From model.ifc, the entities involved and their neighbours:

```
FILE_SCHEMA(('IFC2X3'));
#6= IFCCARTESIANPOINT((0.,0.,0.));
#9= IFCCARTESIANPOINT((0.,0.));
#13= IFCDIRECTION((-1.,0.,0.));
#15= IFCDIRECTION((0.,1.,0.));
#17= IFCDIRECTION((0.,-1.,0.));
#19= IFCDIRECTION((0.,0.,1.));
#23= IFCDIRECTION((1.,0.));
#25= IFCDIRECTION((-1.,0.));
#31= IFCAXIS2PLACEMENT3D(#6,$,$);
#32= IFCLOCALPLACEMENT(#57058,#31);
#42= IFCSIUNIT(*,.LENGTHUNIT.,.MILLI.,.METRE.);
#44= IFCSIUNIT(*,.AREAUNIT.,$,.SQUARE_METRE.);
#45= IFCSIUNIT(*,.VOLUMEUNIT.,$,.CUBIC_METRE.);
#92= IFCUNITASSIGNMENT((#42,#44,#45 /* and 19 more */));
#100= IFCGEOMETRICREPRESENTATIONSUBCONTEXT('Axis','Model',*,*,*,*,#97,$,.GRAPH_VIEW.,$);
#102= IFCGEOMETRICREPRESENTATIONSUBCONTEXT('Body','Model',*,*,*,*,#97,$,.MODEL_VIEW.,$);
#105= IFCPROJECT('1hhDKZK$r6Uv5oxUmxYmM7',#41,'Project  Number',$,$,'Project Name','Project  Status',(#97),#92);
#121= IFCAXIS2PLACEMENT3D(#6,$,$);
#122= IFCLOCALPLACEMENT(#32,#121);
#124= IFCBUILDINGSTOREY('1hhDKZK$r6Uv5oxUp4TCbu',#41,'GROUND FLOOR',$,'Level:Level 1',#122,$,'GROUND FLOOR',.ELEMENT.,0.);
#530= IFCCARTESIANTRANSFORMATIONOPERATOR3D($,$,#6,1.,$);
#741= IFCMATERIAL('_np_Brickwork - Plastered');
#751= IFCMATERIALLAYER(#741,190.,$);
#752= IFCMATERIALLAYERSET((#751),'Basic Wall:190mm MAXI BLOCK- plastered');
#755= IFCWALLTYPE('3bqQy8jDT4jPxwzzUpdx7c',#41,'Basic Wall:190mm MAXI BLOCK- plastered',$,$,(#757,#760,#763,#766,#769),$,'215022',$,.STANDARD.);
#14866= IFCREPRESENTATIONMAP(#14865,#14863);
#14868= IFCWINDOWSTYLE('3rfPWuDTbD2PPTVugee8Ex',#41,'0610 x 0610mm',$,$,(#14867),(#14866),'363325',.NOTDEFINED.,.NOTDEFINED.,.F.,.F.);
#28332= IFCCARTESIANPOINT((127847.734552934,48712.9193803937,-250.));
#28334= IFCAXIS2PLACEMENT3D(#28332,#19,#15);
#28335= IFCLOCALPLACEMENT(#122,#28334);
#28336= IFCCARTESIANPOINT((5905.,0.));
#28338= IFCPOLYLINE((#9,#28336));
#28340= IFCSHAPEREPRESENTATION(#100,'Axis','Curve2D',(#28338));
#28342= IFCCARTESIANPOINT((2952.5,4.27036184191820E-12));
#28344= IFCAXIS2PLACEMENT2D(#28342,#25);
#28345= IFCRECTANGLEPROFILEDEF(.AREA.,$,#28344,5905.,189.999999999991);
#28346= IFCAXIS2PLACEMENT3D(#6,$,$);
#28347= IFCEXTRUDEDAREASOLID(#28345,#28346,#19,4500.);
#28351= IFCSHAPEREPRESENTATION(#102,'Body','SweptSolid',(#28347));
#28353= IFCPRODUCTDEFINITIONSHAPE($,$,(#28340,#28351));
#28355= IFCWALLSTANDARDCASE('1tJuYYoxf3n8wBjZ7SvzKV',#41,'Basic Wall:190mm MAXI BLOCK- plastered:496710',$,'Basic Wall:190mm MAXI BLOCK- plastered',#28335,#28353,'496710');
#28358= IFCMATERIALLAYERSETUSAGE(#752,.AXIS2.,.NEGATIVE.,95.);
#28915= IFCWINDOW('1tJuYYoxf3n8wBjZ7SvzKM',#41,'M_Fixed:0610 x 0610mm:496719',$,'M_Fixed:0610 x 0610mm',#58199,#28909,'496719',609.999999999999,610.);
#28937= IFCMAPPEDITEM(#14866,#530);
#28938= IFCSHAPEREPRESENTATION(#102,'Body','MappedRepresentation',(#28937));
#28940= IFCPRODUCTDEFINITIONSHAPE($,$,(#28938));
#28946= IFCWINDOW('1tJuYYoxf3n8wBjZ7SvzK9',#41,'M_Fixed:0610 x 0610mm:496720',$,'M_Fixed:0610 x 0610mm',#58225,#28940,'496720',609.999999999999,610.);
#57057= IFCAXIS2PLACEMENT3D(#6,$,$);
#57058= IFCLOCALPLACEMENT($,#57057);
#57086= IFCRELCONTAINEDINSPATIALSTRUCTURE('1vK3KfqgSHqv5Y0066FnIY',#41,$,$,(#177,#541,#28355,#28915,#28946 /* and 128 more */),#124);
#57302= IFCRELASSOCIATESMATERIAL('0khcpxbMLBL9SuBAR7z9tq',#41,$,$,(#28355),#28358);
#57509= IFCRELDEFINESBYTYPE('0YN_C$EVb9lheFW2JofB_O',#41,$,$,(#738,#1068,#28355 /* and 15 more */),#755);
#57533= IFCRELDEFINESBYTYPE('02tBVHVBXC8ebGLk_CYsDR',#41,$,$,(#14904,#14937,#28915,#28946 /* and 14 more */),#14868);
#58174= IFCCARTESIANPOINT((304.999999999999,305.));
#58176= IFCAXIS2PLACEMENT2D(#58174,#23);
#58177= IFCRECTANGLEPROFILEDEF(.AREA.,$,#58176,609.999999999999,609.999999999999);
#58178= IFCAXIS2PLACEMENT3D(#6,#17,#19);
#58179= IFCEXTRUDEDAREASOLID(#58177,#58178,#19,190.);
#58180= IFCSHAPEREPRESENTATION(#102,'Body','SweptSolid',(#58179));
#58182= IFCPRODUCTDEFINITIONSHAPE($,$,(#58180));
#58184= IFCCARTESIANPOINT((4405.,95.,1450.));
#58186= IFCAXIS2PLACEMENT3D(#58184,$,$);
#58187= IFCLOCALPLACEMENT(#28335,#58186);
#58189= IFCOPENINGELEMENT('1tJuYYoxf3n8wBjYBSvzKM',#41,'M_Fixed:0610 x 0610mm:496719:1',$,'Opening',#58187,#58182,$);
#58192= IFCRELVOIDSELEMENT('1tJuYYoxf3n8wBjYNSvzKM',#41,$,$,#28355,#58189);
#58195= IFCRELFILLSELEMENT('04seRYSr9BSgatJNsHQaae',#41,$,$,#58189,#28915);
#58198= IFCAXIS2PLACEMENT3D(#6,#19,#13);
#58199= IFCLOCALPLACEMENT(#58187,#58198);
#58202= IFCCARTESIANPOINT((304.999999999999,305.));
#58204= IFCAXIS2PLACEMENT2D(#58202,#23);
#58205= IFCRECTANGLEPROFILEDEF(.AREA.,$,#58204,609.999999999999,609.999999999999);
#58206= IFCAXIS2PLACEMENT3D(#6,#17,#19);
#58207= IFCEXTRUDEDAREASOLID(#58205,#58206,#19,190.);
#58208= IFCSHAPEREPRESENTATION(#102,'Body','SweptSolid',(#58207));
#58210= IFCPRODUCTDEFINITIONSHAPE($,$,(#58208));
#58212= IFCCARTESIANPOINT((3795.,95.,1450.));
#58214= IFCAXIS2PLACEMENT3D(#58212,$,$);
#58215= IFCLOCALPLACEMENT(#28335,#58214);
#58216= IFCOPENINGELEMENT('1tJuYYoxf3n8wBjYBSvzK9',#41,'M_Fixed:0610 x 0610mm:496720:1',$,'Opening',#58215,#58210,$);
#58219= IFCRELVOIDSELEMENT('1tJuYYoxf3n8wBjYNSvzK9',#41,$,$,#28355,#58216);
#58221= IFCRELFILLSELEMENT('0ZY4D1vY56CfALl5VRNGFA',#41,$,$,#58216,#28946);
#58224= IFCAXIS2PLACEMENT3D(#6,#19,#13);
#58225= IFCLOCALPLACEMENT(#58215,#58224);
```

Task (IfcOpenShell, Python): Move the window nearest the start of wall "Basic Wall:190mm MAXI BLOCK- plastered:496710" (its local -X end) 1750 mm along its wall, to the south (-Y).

```python
import ifcopenshell
import ifcopenshell.api.geometry
import ifcopenshell.util.placement
import ifcopenshell.util.unit

model = ifcopenshell.open("model.ifc")
unit_scale = ifcopenshell.util.unit.calculate_unit_scale(model)

window = model.by_id(28946)
opening = window.FillsVoids[0].RelatingOpeningElement
wall = opening.VoidsElements[0].RelatingBuildingElement

wall_matrix = ifcopenshell.util.placement.get_local_placement(wall.ObjectPlacement)
shift = wall_matrix[:3, 0] * -1.75 / unit_scale
before = ifcopenshell.util.placement.get_local_placement(window.ObjectPlacement)[:3, 3].copy()

# The window is placed relative to its opening, so it follows when the opening moves.
matrix = ifcopenshell.util.placement.get_local_placement(opening.ObjectPlacement)
matrix[:3, 3] += shift
ifcopenshell.api.geometry.edit_object_placement(
    model, product=opening, matrix=matrix, is_si=False, should_transform_children=True
)

after = ifcopenshell.util.placement.get_local_placement(window.ObjectPlacement)[:3, 3]
print("window moved by", (after - before).round(3) + 0.0)

model.write("model_edited.ifc")
```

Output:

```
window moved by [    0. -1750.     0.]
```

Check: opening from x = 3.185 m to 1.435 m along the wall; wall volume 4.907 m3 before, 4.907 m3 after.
